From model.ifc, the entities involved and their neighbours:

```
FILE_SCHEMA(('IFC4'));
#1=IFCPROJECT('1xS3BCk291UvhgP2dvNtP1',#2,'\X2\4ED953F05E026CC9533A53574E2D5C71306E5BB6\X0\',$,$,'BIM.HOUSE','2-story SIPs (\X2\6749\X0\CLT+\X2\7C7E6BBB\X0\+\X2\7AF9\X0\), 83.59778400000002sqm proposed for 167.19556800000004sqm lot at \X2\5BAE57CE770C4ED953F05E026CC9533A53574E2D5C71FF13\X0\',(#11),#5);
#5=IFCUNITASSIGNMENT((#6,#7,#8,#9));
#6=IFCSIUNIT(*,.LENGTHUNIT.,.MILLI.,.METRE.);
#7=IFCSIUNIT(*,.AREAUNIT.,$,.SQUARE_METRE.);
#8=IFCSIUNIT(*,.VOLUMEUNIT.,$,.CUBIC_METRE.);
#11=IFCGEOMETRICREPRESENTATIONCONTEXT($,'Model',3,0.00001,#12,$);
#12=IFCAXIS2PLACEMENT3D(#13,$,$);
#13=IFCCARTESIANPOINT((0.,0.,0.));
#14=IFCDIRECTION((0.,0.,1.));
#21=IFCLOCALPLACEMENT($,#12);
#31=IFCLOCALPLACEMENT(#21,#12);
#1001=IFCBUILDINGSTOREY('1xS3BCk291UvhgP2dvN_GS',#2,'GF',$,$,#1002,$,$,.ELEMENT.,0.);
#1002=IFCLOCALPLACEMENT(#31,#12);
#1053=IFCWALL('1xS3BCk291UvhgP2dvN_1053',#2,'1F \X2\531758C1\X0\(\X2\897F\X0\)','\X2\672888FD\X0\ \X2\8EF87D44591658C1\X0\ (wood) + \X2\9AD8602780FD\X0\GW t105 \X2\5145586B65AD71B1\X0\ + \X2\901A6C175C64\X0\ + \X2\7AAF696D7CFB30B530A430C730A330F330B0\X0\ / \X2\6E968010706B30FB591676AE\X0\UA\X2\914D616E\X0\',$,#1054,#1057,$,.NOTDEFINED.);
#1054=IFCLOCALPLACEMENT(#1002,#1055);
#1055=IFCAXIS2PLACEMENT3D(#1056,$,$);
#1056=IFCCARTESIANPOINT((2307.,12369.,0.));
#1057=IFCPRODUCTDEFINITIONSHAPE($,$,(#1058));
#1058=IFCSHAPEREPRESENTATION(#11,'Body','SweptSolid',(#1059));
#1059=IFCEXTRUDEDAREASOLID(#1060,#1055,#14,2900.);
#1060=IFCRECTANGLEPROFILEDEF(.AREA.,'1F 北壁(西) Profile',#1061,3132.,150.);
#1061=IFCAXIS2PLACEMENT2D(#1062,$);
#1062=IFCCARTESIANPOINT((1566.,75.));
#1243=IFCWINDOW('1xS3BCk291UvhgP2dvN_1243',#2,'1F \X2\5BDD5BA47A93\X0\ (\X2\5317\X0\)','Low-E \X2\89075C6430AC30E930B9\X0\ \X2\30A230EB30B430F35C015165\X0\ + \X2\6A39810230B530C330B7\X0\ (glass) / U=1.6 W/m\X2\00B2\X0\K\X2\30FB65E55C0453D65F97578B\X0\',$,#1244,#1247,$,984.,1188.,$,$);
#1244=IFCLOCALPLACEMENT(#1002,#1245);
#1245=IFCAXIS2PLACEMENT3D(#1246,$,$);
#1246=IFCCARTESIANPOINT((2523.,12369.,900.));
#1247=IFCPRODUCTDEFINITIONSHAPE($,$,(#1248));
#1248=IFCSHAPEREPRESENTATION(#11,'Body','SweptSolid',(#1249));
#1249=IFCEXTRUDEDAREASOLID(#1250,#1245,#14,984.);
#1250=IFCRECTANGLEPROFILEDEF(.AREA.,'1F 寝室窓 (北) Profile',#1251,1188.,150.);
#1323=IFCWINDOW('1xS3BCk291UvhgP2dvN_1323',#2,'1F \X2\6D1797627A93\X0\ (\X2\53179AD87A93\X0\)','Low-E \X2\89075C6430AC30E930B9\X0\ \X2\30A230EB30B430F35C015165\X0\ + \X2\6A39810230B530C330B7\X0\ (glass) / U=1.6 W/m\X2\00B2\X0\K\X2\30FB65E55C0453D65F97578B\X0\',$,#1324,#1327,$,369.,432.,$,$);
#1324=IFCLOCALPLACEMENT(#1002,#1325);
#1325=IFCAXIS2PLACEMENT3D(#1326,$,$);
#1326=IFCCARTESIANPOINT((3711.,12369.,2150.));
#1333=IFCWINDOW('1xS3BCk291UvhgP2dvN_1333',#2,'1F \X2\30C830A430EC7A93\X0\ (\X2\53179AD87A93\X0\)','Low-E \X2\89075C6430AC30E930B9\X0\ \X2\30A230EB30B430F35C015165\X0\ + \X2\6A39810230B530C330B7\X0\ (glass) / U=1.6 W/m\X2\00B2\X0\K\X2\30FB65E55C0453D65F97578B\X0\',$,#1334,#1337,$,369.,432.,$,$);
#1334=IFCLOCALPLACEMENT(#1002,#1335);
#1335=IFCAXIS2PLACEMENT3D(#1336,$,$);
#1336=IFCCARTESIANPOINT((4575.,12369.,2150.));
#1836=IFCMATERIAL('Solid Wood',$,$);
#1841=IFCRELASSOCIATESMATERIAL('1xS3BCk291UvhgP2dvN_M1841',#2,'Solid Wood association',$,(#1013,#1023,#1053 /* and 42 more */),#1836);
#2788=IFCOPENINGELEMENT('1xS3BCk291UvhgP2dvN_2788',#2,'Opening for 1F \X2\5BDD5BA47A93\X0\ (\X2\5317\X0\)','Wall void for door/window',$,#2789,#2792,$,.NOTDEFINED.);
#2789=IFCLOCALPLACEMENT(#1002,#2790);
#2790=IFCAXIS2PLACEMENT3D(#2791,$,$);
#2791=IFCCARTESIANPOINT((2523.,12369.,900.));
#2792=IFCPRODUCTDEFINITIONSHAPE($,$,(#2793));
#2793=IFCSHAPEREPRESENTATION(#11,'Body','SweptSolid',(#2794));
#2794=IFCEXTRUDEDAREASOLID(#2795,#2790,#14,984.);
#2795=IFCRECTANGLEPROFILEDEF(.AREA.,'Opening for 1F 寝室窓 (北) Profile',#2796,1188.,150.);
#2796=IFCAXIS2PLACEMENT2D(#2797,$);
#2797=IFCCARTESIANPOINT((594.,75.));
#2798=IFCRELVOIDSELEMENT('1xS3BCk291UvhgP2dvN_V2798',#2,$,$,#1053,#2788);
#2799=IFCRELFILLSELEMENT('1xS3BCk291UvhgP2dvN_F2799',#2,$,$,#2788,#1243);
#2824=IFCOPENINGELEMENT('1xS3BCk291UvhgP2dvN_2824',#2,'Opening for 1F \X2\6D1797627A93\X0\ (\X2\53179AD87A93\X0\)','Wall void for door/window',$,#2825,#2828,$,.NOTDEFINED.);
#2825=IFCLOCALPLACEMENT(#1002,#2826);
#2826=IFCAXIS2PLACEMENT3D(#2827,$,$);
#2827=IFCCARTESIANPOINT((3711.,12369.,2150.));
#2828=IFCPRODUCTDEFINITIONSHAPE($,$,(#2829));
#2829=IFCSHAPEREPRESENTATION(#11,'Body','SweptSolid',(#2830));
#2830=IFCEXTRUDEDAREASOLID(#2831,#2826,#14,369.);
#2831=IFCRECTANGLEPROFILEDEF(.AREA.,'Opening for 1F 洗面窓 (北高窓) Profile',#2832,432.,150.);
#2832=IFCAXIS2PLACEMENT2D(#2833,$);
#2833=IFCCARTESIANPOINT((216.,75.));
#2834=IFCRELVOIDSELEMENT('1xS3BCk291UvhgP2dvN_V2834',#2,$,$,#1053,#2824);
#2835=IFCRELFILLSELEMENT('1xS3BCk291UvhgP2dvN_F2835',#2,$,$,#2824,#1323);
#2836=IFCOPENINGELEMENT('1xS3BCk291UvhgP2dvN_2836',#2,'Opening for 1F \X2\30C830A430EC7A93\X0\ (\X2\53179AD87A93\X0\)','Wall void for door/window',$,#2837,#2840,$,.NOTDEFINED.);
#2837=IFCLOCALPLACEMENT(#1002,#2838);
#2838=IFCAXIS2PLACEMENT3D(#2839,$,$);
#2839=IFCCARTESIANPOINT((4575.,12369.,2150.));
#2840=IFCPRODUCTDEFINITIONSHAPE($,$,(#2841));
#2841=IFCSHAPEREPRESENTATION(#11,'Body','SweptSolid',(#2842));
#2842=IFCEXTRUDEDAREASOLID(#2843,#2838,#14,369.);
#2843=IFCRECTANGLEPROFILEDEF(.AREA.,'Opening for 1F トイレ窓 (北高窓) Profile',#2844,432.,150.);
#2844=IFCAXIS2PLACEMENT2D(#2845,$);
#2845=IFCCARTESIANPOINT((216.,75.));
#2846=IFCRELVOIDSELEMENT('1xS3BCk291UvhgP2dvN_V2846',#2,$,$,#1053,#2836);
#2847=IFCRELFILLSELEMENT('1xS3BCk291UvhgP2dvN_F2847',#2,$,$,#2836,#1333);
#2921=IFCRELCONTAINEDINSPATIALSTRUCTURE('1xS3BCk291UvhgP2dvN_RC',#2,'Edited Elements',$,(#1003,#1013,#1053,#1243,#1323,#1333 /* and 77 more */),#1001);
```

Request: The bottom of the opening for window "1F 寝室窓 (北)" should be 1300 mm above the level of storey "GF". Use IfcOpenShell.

```python
import numpy as np
import ifcopenshell
import ifcopenshell.api.geometry
import ifcopenshell.geom
import ifcopenshell.util.element
import ifcopenshell.util.placement
import ifcopenshell.util.shape
import ifcopenshell.util.unit

model = ifcopenshell.open("model.ifc")
unit_scale = ifcopenshell.util.unit.calculate_unit_scale(model)

window = model.by_guid("1xS3BCk291UvhgP2dvN_1243")
opening = window.FillsVoids[0].RelatingOpeningElement
storey = ifcopenshell.util.element.get_container(window, ifc_class="IfcBuildingStorey")
level = ifcopenshell.util.placement.get_local_placement(storey.ObjectPlacement)[2, 3]

# The opening's origin need not be at the sill, so measure its lowest point.
shape = ifcopenshell.geom.create_shape(ifcopenshell.geom.settings(), opening)
bottom = ifcopenshell.util.shape.get_shape_bottom_elevation(shape, shape.geometry) / unit_scale
dz = level + 1.3 / unit_scale - bottom

shift = np.array([0.0, 0.0, dz])
# The window is not placed relative to its opening, so move both.
for product in (opening, window):
    matrix = ifcopenshell.util.placement.get_local_placement(product.ObjectPlacement)
    matrix[:3, 3] += shift
    ifcopenshell.api.geometry.edit_object_placement(model, product=product, matrix=matrix, is_si=False)

print(f"moved by {dz * unit_scale:+.3f} m")

model.write("model_edited.ifc")
```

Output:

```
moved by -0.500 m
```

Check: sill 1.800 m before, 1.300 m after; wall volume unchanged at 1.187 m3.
